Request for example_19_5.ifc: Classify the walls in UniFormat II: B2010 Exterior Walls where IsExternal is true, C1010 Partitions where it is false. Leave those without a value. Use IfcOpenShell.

First a look at what the model holds.

```python
import ifcopenshell
import ifcopenshell.util.element

model = ifcopenshell.open("example_19_5.ifc")
print(model.schema)
print("classifications:", [c.Name for c in model.by_type("IfcClassification")])
values = [ifcopenshell.util.element.get_pset(e, "Pset_WallCommon", "IsExternal") for e in model.by_type("IfcWall")]
for value in (True, False, None):
    print("IsExternal", value, values.count(value))
```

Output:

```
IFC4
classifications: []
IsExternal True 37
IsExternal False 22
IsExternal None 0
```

```python
import ifcopenshell
import ifcopenshell.api.classification
import ifcopenshell.util.element

model = ifcopenshell.open("example_19_5.ifc")

system = ifcopenshell.api.classification.add_classification(model, classification="UniFormat II")

walls = model.by_type("IfcWall")
external = {e: ifcopenshell.util.element.get_pset(e, "Pset_WallCommon", "IsExternal") for e in walls}
for flag, code, name in ((True, "B2010", "Exterior Walls"), (False, "C1010", "Partitions")):
    products = [e for e in walls if external[e] is flag]
    ifcopenshell.api.classification.add_reference(
        model, products=products, classification=system, identification=code, name=name
    )
    print(code, len(products))

model.write("example_19_5_v2.ifc")
```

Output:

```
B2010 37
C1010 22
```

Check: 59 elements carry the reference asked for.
